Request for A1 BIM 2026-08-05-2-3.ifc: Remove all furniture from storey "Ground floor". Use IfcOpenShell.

First a look at what the model holds.

```python
import ifcopenshell
import ifcopenshell.util.element

model = ifcopenshell.open("A1 BIM 2026-08-05-2-3.ifc")
print(model.schema)
storey = next(s for s in model.by_type("IfcBuildingStorey") if s.Name == "Ground floor")
furniture = [e for e in ifcopenshell.util.element.get_decomposition(storey) if e.is_a("IfcFurnishingElement")]
seen = {}
for e in furniture:
    element_type = ifcopenshell.util.element.get_type(e)
    name = element_type.Name if element_type not in (None, e) else None
    seen[name] = seen.get(name, 0) + 1
for name, count in sorted(seen.items(), key=str):
    print(count, "x", name)
```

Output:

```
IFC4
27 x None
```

```python
import ifcopenshell
import ifcopenshell.api.root
import ifcopenshell.util.element

model = ifcopenshell.open("A1 BIM 2026-08-05-2-3.ifc")

storey = next(s for s in model.by_type("IfcBuildingStorey") if s.Name == "Ground floor")
furniture = [e for e in ifcopenshell.util.element.get_decomposition(storey) if e.is_a("IfcFurnishingElement")]

for e in furniture:
    ifcopenshell.api.root.remove_product(model, product=e)
print(len(furniture), "removed")

model.write("A1 BIM 2026-08-05-2-3_v2.ifc")
```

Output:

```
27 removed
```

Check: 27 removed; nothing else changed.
